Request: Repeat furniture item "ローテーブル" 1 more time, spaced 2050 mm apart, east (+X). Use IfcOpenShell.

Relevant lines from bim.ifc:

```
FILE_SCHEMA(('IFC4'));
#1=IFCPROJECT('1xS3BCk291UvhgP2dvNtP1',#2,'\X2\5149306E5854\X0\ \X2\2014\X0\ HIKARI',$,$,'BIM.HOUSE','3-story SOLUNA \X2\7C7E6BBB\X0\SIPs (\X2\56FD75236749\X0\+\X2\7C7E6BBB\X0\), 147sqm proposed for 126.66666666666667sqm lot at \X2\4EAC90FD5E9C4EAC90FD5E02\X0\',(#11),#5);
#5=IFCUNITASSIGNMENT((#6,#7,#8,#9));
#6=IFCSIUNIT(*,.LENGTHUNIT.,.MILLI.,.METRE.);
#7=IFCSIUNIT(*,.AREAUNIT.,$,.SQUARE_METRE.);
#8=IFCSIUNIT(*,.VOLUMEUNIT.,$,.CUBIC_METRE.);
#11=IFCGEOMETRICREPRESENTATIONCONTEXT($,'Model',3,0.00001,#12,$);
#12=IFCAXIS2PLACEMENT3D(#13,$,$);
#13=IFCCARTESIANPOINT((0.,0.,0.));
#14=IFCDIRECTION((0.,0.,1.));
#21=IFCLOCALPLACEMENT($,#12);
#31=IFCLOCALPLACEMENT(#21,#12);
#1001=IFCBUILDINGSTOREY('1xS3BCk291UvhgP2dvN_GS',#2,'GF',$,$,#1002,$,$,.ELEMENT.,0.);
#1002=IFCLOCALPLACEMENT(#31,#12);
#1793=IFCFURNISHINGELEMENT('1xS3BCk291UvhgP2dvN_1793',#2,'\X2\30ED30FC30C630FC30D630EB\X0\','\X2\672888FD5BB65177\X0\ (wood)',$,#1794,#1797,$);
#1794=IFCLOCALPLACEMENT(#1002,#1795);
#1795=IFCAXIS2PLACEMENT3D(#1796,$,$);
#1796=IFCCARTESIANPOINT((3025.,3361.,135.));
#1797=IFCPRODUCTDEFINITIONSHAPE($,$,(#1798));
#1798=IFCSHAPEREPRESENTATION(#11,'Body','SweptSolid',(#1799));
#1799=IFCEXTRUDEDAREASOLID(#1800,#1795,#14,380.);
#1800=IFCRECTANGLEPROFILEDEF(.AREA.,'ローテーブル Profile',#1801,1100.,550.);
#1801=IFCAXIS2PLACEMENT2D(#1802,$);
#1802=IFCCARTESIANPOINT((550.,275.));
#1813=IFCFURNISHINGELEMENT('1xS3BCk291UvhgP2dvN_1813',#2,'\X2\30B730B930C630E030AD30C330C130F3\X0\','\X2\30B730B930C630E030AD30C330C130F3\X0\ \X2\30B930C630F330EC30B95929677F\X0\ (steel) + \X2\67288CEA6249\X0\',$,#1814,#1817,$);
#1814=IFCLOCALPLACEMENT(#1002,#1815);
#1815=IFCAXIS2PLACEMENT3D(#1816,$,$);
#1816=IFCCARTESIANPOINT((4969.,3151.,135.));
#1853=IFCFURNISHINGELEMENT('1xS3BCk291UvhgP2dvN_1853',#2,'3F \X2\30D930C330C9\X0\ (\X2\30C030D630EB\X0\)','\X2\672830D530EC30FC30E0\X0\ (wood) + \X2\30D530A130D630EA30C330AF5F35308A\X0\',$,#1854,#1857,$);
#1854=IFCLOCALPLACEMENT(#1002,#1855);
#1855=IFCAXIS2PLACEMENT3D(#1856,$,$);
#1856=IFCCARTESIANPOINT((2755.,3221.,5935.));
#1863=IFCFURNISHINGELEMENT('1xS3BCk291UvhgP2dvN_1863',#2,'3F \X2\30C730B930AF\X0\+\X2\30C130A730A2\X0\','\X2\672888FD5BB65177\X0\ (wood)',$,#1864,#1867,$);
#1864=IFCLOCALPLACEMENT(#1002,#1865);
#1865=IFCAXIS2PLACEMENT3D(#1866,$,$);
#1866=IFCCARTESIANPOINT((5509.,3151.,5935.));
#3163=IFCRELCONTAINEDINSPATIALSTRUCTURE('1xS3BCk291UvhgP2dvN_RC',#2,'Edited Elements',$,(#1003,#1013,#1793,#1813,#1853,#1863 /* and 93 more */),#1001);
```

```python
import numpy as np
import ifcopenshell
import ifcopenshell.api.geometry
import ifcopenshell.api.root
import ifcopenshell.util.element
import ifcopenshell.util.placement
import ifcopenshell.util.unit

model = ifcopenshell.open("bim.ifc")
unit_scale = ifcopenshell.util.unit.calculate_unit_scale(model)


def reuse_history(source, copy):
    """copy_class also copies each property set's owner history, people and application; keep the originals."""
    for rel in copy.IsDefinedBy:
        if rel.is_a("IfcRelDefinesByProperties") and (history := rel.RelatingPropertyDefinition.OwnerHistory):
            rel.RelatingPropertyDefinition.OwnerHistory = source.OwnerHistory
            ifcopenshell.util.element.remove_deep2(model, history)


source = model.by_id(1793)
base = ifcopenshell.util.placement.get_local_placement(source.ObjectPlacement)
step = np.array([1.0, 0.0, 0.0]) * 2.05 / unit_scale

for i in range(1, 2):
    copy = ifcopenshell.api.root.copy_class(model, product=source)
    copy.Representation = ifcopenshell.util.element.copy_deep(
        model, source.Representation, exclude=["IfcGeometricRepresentationContext", "IfcRepresentationMap"]
    )
    reuse_history(source, copy)
    matrix = base.copy()
    matrix[:3, 3] += i * step
    print("added at", matrix[:3, 3].round(3) + 0.0)
    ifcopenshell.api.geometry.edit_object_placement(model, product=copy, matrix=matrix, is_si=False)

model.write("bim_edited.ifc")
```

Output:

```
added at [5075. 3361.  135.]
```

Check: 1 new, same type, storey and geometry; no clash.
